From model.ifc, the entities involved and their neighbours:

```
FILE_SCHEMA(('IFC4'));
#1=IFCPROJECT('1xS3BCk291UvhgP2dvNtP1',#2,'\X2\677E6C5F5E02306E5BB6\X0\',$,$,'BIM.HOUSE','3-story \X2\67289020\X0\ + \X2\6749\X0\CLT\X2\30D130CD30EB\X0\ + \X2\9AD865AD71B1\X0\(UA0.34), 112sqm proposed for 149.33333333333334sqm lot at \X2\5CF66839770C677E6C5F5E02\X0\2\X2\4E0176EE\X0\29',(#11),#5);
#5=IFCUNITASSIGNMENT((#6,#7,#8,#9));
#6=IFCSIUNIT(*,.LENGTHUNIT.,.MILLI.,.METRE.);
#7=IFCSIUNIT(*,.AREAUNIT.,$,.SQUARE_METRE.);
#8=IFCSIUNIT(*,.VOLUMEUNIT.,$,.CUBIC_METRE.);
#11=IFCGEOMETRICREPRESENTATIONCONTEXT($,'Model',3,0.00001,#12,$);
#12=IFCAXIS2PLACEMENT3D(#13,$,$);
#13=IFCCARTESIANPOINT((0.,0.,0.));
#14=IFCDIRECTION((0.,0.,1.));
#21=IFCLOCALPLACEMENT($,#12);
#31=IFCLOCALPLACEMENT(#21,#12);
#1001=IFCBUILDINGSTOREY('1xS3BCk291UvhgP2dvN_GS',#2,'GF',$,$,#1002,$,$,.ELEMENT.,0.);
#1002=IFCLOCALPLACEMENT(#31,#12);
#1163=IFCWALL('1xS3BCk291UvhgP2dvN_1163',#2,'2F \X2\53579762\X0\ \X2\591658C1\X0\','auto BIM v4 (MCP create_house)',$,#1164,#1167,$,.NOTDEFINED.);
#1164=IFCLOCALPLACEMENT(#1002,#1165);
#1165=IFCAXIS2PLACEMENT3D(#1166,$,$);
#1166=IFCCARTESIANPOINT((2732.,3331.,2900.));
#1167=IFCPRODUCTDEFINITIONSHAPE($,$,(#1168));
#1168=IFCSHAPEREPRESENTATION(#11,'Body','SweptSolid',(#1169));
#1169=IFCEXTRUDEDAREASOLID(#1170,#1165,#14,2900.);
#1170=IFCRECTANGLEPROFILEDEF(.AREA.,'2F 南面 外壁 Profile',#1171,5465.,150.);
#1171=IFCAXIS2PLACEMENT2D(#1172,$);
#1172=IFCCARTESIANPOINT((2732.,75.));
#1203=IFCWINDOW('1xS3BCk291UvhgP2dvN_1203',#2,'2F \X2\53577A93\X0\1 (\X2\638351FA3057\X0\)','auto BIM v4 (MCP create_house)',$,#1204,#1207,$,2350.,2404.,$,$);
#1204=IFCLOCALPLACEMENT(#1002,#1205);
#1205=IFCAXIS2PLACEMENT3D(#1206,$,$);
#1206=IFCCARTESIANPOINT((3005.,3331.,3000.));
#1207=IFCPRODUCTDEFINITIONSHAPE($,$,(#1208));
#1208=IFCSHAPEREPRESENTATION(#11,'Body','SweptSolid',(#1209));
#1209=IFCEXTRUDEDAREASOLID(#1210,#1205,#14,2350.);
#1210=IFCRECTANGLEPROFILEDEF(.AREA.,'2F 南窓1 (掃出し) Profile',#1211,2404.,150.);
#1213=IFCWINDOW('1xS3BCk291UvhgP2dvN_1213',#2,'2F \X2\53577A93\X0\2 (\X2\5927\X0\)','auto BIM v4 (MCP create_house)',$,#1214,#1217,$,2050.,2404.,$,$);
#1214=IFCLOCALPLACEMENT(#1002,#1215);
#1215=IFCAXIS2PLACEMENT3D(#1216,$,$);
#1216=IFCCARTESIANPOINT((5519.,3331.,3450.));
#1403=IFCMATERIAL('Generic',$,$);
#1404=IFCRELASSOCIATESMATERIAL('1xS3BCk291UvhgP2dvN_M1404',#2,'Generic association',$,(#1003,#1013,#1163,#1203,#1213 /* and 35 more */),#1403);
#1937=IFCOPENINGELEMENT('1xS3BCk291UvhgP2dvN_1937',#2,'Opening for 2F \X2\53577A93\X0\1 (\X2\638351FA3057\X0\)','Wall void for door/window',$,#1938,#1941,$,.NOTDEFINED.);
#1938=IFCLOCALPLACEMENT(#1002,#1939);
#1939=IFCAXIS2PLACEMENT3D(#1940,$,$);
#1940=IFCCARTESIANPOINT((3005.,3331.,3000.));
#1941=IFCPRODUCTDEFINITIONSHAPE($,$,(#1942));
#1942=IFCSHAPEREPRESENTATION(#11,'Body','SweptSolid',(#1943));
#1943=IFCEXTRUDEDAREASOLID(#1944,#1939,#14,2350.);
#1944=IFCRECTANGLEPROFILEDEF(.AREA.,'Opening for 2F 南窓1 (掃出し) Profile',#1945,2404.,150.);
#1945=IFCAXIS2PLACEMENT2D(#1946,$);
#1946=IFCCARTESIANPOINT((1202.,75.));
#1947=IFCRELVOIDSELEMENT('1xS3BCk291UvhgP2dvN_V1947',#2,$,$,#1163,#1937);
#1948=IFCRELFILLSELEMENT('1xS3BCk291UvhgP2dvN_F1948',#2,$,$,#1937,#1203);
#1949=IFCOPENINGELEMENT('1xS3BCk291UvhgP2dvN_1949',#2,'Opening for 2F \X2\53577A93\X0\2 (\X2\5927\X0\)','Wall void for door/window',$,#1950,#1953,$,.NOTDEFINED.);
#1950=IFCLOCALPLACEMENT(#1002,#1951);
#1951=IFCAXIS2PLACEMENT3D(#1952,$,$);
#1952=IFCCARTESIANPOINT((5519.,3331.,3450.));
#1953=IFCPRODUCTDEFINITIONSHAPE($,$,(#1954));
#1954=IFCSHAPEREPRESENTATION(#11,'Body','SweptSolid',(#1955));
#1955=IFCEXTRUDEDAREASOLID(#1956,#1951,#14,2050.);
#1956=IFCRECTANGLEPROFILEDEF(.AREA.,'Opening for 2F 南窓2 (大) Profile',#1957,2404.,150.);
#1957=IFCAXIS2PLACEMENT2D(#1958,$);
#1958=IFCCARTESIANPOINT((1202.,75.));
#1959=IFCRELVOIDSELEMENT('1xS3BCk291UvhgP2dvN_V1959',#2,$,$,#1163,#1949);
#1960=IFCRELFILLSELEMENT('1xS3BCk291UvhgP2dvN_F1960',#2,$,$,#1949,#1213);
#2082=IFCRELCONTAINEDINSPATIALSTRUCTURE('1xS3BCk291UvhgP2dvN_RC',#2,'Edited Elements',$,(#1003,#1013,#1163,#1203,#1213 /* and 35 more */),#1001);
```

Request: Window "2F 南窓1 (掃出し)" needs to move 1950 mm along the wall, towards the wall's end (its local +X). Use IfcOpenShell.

```python
import ifcopenshell
import ifcopenshell.api.geometry
import ifcopenshell.util.placement

model = ifcopenshell.open("model.ifc")

window = model.by_id(1203)
opening = window.FillsVoids[0].RelatingOpeningElement
wall = opening.VoidsElements[0].RelatingBuildingElement

wall_matrix = ifcopenshell.util.placement.get_local_placement(wall.ObjectPlacement)
shift = wall_matrix[:3, 0] * 1950.0
before = ifcopenshell.util.placement.get_local_placement(window.ObjectPlacement)[:3, 3].copy()

# The window is not placed relative to its opening, so move both.
for product in (opening, window):
    matrix = ifcopenshell.util.placement.get_local_placement(product.ObjectPlacement)
    matrix[:3, 3] += shift
    ifcopenshell.api.geometry.edit_object_placement(model, product=product, matrix=matrix, is_si=False)

after = ifcopenshell.util.placement.get_local_placement(window.ObjectPlacement)[:3, 3]
print("window moved by", (after - before).round(3) + 0.0)

model.write("model_rev.ifc")
```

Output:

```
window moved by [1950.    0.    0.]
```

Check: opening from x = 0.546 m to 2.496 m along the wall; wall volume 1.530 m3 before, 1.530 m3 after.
